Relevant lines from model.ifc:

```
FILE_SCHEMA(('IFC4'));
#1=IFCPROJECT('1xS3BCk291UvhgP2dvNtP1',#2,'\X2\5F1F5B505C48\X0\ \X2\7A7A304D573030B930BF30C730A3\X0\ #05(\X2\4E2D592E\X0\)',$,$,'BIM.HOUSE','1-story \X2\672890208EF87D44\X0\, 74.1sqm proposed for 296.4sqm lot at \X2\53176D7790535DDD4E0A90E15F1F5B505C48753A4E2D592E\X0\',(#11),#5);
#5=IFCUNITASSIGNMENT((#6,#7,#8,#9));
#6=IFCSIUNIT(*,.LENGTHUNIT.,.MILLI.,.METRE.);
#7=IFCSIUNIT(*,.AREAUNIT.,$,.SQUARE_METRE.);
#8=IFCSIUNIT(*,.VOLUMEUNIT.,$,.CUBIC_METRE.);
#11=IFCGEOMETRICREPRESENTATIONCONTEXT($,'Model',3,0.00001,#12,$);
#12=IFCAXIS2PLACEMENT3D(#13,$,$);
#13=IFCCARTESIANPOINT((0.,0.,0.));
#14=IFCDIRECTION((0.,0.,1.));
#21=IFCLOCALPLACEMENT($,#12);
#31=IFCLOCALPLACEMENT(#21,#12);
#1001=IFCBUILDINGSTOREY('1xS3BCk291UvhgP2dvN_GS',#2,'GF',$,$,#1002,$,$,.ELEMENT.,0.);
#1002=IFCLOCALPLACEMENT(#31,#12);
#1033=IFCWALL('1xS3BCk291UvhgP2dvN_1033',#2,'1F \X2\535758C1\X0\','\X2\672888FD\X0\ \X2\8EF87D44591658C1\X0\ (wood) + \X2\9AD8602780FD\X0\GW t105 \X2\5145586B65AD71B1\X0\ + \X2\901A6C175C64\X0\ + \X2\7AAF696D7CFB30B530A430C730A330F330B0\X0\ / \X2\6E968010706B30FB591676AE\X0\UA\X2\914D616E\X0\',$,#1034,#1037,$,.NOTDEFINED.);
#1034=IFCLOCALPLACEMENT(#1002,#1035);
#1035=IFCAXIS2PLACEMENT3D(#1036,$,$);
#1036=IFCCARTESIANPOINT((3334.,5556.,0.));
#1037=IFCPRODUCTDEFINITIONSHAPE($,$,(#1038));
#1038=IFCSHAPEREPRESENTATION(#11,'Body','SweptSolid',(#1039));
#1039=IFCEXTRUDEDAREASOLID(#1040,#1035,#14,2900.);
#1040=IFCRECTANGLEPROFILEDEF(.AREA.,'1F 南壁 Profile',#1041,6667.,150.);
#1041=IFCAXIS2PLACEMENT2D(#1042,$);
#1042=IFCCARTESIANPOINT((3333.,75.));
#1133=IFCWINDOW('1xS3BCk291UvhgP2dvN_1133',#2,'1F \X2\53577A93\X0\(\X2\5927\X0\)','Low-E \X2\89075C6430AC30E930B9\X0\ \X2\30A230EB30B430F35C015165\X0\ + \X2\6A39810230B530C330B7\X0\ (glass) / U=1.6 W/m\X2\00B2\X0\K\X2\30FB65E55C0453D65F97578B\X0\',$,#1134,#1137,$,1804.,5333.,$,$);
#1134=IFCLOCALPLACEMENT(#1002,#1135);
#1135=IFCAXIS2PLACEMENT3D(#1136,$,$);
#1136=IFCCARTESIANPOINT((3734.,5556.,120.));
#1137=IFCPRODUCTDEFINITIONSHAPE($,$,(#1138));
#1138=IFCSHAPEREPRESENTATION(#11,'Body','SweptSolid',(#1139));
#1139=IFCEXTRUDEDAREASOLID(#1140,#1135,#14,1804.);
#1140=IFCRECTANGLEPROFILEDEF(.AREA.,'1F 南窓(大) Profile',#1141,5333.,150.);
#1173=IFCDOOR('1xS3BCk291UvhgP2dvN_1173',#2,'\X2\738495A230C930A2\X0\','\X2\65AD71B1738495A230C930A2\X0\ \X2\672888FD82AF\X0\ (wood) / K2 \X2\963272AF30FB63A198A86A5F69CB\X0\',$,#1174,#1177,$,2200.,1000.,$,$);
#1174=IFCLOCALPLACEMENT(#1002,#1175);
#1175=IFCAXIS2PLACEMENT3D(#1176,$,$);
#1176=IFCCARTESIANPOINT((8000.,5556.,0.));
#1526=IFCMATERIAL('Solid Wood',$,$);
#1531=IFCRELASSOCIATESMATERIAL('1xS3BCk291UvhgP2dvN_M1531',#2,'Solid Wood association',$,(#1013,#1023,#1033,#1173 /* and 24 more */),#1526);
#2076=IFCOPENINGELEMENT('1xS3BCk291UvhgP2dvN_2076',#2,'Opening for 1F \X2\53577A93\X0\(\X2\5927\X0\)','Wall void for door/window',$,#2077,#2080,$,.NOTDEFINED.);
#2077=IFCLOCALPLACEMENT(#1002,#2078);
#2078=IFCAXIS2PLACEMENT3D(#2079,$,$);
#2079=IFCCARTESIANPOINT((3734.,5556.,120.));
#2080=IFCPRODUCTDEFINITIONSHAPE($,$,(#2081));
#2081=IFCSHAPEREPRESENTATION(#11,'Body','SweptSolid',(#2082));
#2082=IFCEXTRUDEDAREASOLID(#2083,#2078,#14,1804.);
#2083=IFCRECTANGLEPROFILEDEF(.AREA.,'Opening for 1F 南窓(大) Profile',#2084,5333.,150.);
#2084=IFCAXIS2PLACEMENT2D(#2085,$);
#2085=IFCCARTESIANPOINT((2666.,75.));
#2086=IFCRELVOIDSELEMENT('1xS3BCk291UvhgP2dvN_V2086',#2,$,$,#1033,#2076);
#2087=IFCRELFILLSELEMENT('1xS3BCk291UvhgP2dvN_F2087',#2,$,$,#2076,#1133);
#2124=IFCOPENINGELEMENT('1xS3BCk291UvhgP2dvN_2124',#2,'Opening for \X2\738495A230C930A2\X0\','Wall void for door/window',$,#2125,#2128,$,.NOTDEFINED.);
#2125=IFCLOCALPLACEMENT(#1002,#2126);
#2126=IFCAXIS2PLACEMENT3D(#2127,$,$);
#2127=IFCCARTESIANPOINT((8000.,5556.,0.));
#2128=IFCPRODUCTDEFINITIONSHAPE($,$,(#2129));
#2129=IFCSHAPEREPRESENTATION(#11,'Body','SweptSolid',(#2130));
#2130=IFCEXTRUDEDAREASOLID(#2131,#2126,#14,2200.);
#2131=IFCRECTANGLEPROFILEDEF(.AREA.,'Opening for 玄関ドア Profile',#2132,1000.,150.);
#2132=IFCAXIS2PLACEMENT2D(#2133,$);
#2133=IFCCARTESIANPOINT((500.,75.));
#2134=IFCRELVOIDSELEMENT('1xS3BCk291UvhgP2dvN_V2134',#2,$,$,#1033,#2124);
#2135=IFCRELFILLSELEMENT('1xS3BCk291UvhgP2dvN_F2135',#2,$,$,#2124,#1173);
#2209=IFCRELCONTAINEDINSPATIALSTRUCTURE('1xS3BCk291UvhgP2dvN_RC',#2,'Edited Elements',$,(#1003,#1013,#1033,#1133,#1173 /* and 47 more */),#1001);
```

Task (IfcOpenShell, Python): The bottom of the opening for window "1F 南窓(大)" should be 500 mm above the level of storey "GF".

```python
import numpy as np
import ifcopenshell
import ifcopenshell.api.geometry
import ifcopenshell.geom
import ifcopenshell.util.element
import ifcopenshell.util.placement
import ifcopenshell.util.shape
import ifcopenshell.util.unit

model = ifcopenshell.open("model.ifc")
unit_scale = ifcopenshell.util.unit.calculate_unit_scale(model)

window = model.by_id(1133)
opening = window.FillsVoids[0].RelatingOpeningElement
storey = ifcopenshell.util.element.get_container(window, ifc_class="IfcBuildingStorey")
level = ifcopenshell.util.placement.get_local_placement(storey.ObjectPlacement)[2, 3]

# The opening's origin need not be at the sill, so measure its lowest point.
shape = ifcopenshell.geom.create_shape(ifcopenshell.geom.settings(), opening)
bottom = ifcopenshell.util.shape.get_shape_bottom_elevation(shape, shape.geometry) / unit_scale
dz = level + 0.5 / unit_scale - bottom

shift = np.array([0.0, 0.0, dz])
# The window is not placed relative to its opening, so move both.
for product in (opening, window):
    matrix = ifcopenshell.util.placement.get_local_placement(product.ObjectPlacement)
    matrix[:3, 3] += shift
    ifcopenshell.api.geometry.edit_object_placement(model, product=product, matrix=matrix, is_si=False)

print(f"moved by {dz * unit_scale:+.3f} m")

model.write("model_edited.ifc")
```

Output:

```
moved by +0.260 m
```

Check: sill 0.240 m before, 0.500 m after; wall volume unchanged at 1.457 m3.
